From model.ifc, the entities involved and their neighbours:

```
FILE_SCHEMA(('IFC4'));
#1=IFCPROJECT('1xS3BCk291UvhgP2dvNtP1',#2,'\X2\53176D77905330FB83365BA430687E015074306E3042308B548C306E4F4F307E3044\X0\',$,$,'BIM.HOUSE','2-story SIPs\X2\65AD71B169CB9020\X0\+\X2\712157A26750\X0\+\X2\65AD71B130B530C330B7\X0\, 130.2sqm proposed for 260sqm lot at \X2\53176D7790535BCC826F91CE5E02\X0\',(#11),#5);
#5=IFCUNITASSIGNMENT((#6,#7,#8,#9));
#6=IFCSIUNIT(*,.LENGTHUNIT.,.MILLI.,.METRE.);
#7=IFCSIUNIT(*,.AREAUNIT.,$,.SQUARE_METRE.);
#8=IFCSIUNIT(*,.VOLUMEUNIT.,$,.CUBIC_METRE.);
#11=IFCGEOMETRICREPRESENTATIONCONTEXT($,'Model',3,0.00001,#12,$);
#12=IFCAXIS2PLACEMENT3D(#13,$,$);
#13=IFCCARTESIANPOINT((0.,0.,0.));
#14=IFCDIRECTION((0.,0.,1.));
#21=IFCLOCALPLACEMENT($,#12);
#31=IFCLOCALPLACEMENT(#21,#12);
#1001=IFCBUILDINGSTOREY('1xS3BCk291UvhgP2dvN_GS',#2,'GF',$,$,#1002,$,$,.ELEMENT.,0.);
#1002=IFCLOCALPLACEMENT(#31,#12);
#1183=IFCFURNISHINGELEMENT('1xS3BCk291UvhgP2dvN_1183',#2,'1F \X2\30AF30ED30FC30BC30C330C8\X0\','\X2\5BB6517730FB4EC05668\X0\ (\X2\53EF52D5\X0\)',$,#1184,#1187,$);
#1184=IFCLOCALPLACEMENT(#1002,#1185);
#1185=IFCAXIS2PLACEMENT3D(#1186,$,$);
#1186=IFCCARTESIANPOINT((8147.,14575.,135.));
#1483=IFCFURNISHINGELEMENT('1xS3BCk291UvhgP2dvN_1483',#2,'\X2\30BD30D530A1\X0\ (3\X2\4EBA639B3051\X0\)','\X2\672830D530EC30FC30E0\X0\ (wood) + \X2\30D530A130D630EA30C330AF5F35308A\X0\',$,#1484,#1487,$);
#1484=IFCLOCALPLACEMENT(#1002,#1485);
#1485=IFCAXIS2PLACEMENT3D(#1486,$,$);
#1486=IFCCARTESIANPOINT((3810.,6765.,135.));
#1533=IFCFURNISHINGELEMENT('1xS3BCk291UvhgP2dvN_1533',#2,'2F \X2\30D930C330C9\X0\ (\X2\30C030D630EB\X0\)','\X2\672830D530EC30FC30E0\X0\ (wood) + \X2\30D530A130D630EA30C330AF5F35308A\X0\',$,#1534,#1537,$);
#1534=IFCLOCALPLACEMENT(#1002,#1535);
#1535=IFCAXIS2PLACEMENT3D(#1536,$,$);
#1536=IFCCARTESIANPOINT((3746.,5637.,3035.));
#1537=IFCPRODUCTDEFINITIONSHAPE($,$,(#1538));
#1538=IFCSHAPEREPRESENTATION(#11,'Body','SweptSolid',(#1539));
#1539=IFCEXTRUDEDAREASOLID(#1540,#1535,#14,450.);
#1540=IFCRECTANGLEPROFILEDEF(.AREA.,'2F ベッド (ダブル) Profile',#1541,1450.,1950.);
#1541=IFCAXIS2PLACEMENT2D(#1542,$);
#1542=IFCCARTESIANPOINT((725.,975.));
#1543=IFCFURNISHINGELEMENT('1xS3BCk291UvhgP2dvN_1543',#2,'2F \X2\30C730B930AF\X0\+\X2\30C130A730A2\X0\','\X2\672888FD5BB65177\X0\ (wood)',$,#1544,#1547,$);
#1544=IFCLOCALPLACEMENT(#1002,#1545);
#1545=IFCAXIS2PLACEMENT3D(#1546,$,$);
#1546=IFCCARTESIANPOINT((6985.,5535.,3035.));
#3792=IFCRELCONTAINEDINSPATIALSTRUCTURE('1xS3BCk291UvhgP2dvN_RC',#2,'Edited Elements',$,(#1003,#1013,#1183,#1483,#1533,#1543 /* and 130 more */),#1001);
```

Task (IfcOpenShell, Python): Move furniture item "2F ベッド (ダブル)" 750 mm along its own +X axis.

```python
import ifcopenshell
import ifcopenshell.api.geometry
import ifcopenshell.util.placement
import ifcopenshell.util.unit

model = ifcopenshell.open("model.ifc")
unit_scale = ifcopenshell.util.unit.calculate_unit_scale(model)

item = model.by_guid("1xS3BCk291UvhgP2dvN_1533")
matrix = ifcopenshell.util.placement.get_local_placement(item.ObjectPlacement)
matrix[:3, 3] += matrix[:3, 0] * 0.75 / unit_scale
ifcopenshell.api.geometry.edit_object_placement(model, product=item, matrix=matrix, is_si=False)

print(ifcopenshell.util.placement.get_local_placement(item.ObjectPlacement).round(3) + 0.0)

model.write("model_updated.ifc")
```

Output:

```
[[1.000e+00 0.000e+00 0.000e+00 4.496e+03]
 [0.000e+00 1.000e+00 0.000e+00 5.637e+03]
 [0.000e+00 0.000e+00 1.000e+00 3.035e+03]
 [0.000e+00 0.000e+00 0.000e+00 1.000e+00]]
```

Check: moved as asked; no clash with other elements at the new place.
